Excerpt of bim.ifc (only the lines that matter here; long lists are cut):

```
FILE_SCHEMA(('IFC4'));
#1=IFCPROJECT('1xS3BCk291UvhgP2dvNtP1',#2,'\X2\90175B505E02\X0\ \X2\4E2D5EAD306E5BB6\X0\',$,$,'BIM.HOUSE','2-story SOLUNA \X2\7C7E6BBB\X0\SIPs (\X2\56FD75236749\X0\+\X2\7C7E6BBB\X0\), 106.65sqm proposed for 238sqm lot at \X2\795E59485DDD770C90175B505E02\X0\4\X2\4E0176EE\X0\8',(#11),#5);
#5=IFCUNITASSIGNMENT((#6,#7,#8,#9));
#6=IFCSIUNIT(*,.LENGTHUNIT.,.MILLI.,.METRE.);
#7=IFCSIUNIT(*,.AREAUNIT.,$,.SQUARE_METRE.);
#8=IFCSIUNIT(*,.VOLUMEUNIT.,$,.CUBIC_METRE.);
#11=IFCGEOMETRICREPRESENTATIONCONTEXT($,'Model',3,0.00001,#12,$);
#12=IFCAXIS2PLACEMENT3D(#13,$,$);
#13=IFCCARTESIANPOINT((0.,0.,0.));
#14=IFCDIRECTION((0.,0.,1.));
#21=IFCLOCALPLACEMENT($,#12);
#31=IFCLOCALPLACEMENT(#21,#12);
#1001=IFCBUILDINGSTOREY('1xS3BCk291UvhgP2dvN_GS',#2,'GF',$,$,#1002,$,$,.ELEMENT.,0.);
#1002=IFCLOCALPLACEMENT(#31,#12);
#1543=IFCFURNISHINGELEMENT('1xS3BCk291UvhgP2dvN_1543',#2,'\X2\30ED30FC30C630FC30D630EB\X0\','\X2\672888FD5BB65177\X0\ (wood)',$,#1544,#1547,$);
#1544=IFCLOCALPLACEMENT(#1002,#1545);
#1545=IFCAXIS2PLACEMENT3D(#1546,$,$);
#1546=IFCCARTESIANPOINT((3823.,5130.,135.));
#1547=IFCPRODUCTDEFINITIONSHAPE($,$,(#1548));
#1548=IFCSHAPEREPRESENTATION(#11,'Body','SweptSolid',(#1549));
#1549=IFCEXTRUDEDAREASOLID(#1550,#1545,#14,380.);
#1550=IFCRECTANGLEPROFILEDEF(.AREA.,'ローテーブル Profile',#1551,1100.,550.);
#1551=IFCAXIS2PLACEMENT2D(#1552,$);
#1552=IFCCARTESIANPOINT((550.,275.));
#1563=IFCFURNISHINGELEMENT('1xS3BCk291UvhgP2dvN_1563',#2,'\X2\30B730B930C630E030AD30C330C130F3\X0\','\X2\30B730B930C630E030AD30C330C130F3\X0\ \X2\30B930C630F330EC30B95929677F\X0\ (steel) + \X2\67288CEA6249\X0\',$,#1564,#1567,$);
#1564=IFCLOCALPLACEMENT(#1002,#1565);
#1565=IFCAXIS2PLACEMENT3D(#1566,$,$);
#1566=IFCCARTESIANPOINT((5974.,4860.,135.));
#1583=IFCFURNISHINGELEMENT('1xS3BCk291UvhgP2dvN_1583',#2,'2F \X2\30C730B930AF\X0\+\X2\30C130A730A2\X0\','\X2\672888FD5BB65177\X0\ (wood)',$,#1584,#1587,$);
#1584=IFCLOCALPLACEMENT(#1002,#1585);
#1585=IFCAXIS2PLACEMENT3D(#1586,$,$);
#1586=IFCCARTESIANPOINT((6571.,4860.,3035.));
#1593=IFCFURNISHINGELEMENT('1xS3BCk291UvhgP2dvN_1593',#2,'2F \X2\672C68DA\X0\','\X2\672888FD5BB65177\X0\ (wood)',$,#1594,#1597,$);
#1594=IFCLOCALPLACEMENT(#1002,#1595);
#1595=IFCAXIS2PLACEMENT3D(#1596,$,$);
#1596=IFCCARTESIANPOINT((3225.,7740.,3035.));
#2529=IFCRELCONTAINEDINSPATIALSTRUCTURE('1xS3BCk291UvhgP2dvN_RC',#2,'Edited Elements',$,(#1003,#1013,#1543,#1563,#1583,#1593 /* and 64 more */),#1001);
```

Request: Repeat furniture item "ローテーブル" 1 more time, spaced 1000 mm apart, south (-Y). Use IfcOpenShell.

```python
import numpy as np
import ifcopenshell
import ifcopenshell.api.geometry
import ifcopenshell.api.root
import ifcopenshell.util.element
import ifcopenshell.util.placement
import ifcopenshell.util.unit

model = ifcopenshell.open("bim.ifc")
unit_scale = ifcopenshell.util.unit.calculate_unit_scale(model)


def reuse_history(source, copy):
    """copy_class also copies each property set's owner history, people and application; keep the originals."""
    for rel in copy.IsDefinedBy:
        if rel.is_a("IfcRelDefinesByProperties") and (history := rel.RelatingPropertyDefinition.OwnerHistory):
            rel.RelatingPropertyDefinition.OwnerHistory = source.OwnerHistory
            ifcopenshell.util.element.remove_deep2(model, history)


source = model.by_guid("1xS3BCk291UvhgP2dvN_1543")
base = ifcopenshell.util.placement.get_local_placement(source.ObjectPlacement)
step = np.array([0.0, -1.0, 0.0]) * 1 / unit_scale

for i in range(1, 2):
    copy = ifcopenshell.api.root.copy_class(model, product=source)
    copy.Representation = ifcopenshell.util.element.copy_deep(
        model, source.Representation, exclude=["IfcGeometricRepresentationContext", "IfcRepresentationMap"]
    )
    reuse_history(source, copy)
    matrix = base.copy()
    matrix[:3, 3] += i * step
    print("added at", matrix[:3, 3].round(3) + 0.0)
    ifcopenshell.api.geometry.edit_object_placement(model, product=copy, matrix=matrix, is_si=False)

model.write("bim-out.ifc")
```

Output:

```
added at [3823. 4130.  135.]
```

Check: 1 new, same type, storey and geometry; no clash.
